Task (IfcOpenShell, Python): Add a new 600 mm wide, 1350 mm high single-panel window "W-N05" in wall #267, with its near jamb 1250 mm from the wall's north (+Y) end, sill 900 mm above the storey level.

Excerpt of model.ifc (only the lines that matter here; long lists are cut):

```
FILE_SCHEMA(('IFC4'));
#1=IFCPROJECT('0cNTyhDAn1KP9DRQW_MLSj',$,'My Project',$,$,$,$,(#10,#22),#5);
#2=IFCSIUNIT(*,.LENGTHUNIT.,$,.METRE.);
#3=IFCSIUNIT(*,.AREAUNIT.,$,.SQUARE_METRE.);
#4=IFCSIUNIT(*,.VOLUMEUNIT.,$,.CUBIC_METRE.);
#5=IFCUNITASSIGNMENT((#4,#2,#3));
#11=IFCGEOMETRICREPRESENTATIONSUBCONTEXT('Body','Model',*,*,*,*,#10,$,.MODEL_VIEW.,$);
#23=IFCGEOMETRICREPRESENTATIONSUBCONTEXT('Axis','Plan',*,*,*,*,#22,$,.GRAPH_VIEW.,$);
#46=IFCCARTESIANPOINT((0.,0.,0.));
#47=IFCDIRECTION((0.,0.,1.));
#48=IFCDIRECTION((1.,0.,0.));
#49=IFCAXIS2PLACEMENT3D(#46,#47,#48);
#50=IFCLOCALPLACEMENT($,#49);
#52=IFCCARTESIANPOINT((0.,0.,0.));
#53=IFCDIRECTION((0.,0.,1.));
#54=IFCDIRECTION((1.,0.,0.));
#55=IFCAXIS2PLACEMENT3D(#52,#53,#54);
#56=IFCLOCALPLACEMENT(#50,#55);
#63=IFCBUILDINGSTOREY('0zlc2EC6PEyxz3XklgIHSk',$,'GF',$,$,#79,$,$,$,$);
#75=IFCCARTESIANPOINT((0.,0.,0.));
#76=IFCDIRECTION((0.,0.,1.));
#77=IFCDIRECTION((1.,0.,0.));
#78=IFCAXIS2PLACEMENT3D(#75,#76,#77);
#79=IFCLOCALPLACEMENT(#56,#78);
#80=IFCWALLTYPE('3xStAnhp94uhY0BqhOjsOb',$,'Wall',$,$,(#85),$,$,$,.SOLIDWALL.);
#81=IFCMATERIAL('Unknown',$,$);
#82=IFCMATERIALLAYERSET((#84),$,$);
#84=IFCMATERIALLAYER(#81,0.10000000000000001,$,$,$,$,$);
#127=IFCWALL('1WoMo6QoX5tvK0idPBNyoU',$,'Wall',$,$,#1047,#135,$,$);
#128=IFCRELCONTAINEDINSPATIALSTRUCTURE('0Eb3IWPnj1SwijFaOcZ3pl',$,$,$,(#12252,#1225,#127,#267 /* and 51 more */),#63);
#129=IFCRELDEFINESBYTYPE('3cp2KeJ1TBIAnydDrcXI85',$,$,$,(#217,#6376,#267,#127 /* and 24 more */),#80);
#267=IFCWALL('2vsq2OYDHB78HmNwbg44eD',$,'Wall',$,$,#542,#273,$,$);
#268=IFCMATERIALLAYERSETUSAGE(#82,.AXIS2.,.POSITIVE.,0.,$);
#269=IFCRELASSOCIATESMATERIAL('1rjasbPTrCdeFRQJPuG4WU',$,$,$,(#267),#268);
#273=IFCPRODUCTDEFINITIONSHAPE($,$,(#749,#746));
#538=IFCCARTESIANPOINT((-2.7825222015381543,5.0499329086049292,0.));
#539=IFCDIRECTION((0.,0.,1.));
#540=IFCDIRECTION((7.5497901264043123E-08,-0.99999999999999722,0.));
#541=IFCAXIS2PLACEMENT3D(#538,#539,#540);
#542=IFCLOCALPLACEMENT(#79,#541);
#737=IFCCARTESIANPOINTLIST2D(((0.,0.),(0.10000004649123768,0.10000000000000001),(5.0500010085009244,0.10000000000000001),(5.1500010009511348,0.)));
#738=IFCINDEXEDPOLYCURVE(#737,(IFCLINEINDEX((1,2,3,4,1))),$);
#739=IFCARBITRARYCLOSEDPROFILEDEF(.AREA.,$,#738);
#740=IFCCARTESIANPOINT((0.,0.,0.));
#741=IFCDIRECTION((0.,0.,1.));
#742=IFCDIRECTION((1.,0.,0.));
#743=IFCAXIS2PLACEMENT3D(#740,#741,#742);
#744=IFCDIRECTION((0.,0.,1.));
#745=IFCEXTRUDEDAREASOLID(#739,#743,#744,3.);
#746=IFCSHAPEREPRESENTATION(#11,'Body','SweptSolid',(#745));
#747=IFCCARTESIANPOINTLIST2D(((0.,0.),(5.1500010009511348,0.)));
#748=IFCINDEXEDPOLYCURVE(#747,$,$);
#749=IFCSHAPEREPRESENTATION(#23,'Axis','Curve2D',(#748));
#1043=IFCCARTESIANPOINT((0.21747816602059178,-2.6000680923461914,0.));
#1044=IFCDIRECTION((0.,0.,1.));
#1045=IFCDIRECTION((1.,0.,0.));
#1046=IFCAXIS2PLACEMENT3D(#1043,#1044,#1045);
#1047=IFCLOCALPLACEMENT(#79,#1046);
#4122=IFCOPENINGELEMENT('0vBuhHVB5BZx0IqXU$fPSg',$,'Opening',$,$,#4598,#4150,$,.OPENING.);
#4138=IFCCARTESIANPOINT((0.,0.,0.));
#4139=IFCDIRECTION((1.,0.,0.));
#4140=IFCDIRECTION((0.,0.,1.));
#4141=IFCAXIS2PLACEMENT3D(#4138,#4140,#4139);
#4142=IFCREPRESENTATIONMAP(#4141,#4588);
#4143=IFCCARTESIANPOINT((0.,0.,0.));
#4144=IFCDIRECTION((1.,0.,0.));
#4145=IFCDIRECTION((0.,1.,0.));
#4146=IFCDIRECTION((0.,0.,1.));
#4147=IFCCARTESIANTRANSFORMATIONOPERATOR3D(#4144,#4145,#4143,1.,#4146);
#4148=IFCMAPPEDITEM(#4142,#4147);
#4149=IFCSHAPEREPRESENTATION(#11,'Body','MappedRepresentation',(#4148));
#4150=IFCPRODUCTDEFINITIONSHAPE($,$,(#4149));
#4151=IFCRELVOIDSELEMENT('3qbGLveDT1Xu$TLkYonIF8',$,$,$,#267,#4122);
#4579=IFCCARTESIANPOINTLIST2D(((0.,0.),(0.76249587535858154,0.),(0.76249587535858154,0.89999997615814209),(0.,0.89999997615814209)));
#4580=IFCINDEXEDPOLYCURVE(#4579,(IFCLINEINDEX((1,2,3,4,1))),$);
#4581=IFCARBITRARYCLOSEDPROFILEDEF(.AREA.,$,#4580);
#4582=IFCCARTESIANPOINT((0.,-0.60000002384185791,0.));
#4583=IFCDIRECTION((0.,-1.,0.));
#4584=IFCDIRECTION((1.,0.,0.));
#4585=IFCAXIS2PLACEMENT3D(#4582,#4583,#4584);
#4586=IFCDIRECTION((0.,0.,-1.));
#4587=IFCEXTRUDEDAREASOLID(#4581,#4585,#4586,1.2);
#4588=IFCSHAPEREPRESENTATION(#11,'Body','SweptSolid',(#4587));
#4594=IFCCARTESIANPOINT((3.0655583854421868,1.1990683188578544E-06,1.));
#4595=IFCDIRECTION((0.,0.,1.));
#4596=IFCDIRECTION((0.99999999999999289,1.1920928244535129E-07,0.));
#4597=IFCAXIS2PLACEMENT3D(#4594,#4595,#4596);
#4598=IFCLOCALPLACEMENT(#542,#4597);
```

```python
import numpy as np
import ifcopenshell
import ifcopenshell.api.feature
import ifcopenshell.api.geometry
import ifcopenshell.api.root
import ifcopenshell.api.spatial
import ifcopenshell.geom
import ifcopenshell.util.element
import ifcopenshell.util.placement
import ifcopenshell.util.representation
import ifcopenshell.util.shape
import ifcopenshell.util.unit

model = ifcopenshell.open("model.ifc")
unit_scale = ifcopenshell.util.unit.calculate_unit_scale(model)
settings = ifcopenshell.geom.settings()


def volume(element):
    """Net volume in cubic metres, openings subtracted."""
    shape = ifcopenshell.geom.create_shape(settings, element)
    return ifcopenshell.util.shape.get_volume(shape.geometry)


wall = model.by_guid("2vsq2OYDHB78HmNwbg44eD")
storey = ifcopenshell.util.element.get_container(wall, ifc_class="IfcBuildingStorey")
context = ifcopenshell.util.representation.get_context(model, "Model", "Body", "MODEL_VIEW")
before = volume(wall)

width, height, from_end, sill = 0.6, 1.35, 1.25, 0.9  # metres

# The wall runs along its own X axis, and the end named is its -X end.
wall_shape = ifcopenshell.geom.create_shape(settings, wall)
x, y, z = ifcopenshell.util.shape.get_vertices(wall_shape.geometry).T
start = x.min() + from_end
face, thickness = float(y.min()), float(y.max() - y.min())
wall_matrix = ifcopenshell.util.placement.get_local_placement(wall.ObjectPlacement)
level = ifcopenshell.util.placement.get_local_placement(storey.ObjectPlacement)[2, 3]


def in_wall(x, y):
    """Placement at x, y metres in the wall's axes, at sill height."""
    matrix = wall_matrix.copy()
    matrix[:, 3] = wall_matrix @ np.array([x / unit_scale, y / unit_scale, 0.0, 1.0])
    matrix[2, 3] = level + sill / unit_scale
    return matrix


# Opening: a box that overshoots both wall faces by 50 mm.
opening = ifcopenshell.api.root.create_entity(model, ifc_class="IfcOpeningElement", predefined_type="OPENING")
box = ifcopenshell.api.geometry.add_wall_representation(
    model, context=context, length=width, height=height, thickness=thickness + 0.1
)
ifcopenshell.api.geometry.assign_representation(model, product=opening, representation=box)
ifcopenshell.api.geometry.edit_object_placement(model, product=opening, matrix=in_wall(start, face - 0.05), is_si=False)
ifcopenshell.api.feature.add_feature(model, feature=opening, element=wall)

window = ifcopenshell.api.root.create_entity(model, ifc_class="IfcWindow", name="W-N05", predefined_type="WINDOW")
window.OverallWidth, window.OverallHeight = width / unit_scale, height / unit_scale
window.PartitioningType = "SINGLE_PANEL"
body = ifcopenshell.api.geometry.add_window_representation(
    model,
    context=context,
    overall_width=window.OverallWidth,
    overall_height=window.OverallHeight,
    partition_type="SINGLE_PANEL",
)
ifcopenshell.api.geometry.assign_representation(model, product=window, representation=body)
ifcopenshell.api.spatial.assign_container(model, products=[window], relating_structure=storey)
ifcopenshell.api.feature.add_filling(model, opening=opening, element=window)

# Centre the window in the wall's thickness.
ifcopenshell.api.geometry.edit_object_placement(model, product=window, matrix=in_wall(start, face), is_si=False)
window_shape = ifcopenshell.geom.create_shape(settings, window)
depth = ifcopenshell.util.shape.get_vertices(window_shape.geometry)[:, 1]
offset = face + thickness / 2 - (depth.min() + depth.max()) / 2
ifcopenshell.api.geometry.edit_object_placement(model, product=window, matrix=in_wall(start, offset), is_si=False)

after = volume(wall)

print(f"wall volume {before:.3f} -> {after:.3f} m3")

model.write("model-out.ifc")
```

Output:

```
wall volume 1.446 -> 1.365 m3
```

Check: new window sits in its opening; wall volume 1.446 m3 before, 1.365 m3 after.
